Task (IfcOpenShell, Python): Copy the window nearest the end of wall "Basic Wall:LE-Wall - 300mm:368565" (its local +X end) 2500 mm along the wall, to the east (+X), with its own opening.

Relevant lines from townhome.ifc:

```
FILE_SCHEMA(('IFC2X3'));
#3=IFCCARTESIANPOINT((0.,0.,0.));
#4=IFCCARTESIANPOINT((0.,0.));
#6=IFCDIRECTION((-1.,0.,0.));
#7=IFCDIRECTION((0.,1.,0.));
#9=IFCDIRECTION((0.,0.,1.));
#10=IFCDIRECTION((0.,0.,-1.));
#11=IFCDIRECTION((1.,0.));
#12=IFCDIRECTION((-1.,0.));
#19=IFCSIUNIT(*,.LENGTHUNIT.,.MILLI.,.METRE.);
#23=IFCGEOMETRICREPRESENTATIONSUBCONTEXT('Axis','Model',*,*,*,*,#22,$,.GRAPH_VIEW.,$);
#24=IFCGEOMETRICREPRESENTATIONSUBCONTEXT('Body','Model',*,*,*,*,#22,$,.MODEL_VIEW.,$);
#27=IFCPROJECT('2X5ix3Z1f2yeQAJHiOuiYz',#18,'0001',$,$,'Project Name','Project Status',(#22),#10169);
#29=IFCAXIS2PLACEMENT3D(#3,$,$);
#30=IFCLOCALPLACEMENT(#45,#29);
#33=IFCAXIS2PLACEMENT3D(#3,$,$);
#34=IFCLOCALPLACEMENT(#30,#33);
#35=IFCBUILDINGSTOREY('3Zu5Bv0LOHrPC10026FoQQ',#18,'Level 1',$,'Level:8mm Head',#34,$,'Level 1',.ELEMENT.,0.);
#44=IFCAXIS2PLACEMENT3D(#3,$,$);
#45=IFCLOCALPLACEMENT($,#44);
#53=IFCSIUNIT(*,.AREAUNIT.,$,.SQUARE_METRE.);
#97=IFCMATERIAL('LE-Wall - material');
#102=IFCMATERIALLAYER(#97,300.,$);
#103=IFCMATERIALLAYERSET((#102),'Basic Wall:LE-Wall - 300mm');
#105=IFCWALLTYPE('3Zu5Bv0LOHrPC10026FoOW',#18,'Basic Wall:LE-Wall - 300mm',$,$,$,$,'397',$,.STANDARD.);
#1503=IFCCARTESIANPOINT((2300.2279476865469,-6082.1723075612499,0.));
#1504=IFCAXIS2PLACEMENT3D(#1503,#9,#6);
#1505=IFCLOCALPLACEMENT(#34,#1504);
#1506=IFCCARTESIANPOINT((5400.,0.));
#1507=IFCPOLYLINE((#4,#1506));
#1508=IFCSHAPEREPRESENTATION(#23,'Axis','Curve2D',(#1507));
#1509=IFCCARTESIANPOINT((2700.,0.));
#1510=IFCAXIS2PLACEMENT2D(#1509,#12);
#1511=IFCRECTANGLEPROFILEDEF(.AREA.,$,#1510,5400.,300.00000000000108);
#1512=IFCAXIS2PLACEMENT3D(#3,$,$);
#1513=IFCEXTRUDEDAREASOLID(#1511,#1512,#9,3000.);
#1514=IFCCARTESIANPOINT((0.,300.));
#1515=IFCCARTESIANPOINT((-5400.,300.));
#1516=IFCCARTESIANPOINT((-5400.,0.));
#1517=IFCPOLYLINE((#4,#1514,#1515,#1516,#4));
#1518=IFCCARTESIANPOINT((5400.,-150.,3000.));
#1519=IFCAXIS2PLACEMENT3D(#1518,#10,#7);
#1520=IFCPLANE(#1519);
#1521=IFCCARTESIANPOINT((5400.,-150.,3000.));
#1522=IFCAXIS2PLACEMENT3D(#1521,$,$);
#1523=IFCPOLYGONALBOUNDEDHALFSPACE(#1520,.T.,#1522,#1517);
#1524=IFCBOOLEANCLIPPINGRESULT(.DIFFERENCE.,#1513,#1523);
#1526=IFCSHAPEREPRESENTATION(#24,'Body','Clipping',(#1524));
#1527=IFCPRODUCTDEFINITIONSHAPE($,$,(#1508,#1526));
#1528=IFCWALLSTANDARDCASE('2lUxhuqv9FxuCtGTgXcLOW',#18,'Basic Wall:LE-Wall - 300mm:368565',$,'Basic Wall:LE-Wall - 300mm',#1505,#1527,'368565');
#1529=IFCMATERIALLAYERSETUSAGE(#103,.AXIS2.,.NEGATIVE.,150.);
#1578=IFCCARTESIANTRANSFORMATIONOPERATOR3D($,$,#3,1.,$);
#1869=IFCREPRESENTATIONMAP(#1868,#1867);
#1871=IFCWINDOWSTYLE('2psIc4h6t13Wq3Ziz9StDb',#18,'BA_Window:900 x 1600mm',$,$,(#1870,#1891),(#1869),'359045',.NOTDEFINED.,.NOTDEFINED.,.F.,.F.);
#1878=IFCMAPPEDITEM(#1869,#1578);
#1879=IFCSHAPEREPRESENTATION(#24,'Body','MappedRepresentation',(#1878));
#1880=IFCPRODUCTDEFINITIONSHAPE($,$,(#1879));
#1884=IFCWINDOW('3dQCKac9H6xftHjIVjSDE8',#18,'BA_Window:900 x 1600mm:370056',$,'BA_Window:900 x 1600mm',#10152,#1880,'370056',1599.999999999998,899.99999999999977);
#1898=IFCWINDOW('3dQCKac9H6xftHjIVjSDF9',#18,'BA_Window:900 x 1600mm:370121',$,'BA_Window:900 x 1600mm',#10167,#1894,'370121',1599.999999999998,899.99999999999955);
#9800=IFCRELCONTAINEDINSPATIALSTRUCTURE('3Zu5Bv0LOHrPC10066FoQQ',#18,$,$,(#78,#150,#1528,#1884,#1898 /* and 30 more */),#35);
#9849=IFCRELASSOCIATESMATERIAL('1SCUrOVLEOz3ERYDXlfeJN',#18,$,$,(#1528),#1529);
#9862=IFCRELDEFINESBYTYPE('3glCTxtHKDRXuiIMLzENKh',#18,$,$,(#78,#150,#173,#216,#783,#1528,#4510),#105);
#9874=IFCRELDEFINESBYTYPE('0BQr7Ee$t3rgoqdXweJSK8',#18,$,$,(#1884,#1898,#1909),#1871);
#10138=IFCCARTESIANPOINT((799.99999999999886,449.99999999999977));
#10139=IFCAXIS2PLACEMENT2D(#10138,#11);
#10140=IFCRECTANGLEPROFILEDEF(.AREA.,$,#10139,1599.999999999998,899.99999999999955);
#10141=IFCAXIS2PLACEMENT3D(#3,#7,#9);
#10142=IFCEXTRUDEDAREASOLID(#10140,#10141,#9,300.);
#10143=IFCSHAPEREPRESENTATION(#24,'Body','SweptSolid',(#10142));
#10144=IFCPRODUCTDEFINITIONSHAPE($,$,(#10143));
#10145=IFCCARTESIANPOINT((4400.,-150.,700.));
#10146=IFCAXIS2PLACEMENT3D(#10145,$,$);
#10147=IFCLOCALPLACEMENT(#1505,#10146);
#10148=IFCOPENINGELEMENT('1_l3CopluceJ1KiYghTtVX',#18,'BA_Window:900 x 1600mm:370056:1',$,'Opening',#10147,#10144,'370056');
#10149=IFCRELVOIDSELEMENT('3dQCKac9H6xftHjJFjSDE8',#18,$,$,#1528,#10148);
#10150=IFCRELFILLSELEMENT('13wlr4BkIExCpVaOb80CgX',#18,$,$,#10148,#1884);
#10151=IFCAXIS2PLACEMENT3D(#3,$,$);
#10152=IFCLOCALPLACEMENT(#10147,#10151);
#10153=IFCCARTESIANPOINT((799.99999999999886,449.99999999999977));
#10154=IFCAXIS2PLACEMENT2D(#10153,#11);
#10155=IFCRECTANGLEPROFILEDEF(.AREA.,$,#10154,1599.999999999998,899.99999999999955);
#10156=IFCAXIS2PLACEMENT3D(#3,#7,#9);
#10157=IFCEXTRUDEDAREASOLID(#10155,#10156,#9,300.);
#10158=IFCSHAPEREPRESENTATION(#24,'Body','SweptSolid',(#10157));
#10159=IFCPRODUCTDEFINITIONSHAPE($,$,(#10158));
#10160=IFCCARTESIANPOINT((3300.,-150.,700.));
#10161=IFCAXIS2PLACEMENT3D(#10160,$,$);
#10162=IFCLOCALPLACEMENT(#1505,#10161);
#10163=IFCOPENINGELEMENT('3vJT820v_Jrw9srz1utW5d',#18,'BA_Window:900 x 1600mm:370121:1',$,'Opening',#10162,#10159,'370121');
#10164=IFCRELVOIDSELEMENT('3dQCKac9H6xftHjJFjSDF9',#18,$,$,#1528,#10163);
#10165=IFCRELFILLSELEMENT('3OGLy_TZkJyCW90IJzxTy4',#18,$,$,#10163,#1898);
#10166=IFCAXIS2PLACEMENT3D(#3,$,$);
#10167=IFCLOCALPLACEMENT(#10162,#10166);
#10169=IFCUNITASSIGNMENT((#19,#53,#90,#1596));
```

```python
import ifcopenshell
import ifcopenshell.api.feature
import ifcopenshell.api.geometry
import ifcopenshell.api.root
import ifcopenshell.geom
import ifcopenshell.util.element
import ifcopenshell.util.placement
import ifcopenshell.util.shape
import ifcopenshell.util.unit

model = ifcopenshell.open("townhome.ifc")
unit_scale = ifcopenshell.util.unit.calculate_unit_scale(model)
settings = ifcopenshell.geom.settings()


def volume(element):
    """Net volume in cubic metres, openings subtracted."""
    shape = ifcopenshell.geom.create_shape(settings, element)
    return ifcopenshell.util.shape.get_volume(shape.geometry)


def reuse_history(source, copy):
    """copy_class also copies each property set's owner history, people and application; keep the originals."""
    for rel in copy.IsDefinedBy:
        if rel.is_a("IfcRelDefinesByProperties") and (history := rel.RelatingPropertyDefinition.OwnerHistory):
            rel.RelatingPropertyDefinition.OwnerHistory = source.OwnerHistory
            ifcopenshell.util.element.remove_deep2(model, history)


window = model.by_id(1884)
opening = window.FillsVoids[0].RelatingOpeningElement
wall = opening.VoidsElements[0].RelatingBuildingElement
before = volume(wall)
shift = ifcopenshell.util.placement.get_local_placement(wall.ObjectPlacement)[:3, 0] * -2.5 / unit_scale

# copy_class copies the void relationship, type, container and properties, but no geometry.
new_opening = ifcopenshell.api.root.copy_class(model, product=opening)
new_opening.Representation = ifcopenshell.util.element.copy_deep(
    model, opening.Representation, exclude=["IfcGeometricRepresentationContext", "IfcRepresentationMap"]
)
new_opening.Name = "BA_Window:900 x 1600mm"
new_opening.Tag = None
new_window = ifcopenshell.api.root.copy_class(model, product=window)
new_window.Representation = ifcopenshell.util.element.copy_deep(
    model, window.Representation, exclude=["IfcGeometricRepresentationContext", "IfcRepresentationMap"]
)
new_window.Name = "BA_Window:900 x 1600mm"
new_window.Tag = None
reuse_history(window, new_window)
fills = ifcopenshell.api.feature.add_filling(model, opening=new_opening, element=new_window)
fills.OwnerHistory = new_window.OwnerHistory  # required in IFC2X3

for old, new in ((opening, new_opening), (window, new_window)):
    matrix = ifcopenshell.util.placement.get_local_placement(old.ObjectPlacement)
    matrix[:3, 3] += shift
    ifcopenshell.api.geometry.edit_object_placement(model, product=new, matrix=matrix, is_si=False)

after = volume(wall)

print(f"wall volume {before:.3f} -> {after:.3f} m3")

model.write("townhome_rev.ifc")
```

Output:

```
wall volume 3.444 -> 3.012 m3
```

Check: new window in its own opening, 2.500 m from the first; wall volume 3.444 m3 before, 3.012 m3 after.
